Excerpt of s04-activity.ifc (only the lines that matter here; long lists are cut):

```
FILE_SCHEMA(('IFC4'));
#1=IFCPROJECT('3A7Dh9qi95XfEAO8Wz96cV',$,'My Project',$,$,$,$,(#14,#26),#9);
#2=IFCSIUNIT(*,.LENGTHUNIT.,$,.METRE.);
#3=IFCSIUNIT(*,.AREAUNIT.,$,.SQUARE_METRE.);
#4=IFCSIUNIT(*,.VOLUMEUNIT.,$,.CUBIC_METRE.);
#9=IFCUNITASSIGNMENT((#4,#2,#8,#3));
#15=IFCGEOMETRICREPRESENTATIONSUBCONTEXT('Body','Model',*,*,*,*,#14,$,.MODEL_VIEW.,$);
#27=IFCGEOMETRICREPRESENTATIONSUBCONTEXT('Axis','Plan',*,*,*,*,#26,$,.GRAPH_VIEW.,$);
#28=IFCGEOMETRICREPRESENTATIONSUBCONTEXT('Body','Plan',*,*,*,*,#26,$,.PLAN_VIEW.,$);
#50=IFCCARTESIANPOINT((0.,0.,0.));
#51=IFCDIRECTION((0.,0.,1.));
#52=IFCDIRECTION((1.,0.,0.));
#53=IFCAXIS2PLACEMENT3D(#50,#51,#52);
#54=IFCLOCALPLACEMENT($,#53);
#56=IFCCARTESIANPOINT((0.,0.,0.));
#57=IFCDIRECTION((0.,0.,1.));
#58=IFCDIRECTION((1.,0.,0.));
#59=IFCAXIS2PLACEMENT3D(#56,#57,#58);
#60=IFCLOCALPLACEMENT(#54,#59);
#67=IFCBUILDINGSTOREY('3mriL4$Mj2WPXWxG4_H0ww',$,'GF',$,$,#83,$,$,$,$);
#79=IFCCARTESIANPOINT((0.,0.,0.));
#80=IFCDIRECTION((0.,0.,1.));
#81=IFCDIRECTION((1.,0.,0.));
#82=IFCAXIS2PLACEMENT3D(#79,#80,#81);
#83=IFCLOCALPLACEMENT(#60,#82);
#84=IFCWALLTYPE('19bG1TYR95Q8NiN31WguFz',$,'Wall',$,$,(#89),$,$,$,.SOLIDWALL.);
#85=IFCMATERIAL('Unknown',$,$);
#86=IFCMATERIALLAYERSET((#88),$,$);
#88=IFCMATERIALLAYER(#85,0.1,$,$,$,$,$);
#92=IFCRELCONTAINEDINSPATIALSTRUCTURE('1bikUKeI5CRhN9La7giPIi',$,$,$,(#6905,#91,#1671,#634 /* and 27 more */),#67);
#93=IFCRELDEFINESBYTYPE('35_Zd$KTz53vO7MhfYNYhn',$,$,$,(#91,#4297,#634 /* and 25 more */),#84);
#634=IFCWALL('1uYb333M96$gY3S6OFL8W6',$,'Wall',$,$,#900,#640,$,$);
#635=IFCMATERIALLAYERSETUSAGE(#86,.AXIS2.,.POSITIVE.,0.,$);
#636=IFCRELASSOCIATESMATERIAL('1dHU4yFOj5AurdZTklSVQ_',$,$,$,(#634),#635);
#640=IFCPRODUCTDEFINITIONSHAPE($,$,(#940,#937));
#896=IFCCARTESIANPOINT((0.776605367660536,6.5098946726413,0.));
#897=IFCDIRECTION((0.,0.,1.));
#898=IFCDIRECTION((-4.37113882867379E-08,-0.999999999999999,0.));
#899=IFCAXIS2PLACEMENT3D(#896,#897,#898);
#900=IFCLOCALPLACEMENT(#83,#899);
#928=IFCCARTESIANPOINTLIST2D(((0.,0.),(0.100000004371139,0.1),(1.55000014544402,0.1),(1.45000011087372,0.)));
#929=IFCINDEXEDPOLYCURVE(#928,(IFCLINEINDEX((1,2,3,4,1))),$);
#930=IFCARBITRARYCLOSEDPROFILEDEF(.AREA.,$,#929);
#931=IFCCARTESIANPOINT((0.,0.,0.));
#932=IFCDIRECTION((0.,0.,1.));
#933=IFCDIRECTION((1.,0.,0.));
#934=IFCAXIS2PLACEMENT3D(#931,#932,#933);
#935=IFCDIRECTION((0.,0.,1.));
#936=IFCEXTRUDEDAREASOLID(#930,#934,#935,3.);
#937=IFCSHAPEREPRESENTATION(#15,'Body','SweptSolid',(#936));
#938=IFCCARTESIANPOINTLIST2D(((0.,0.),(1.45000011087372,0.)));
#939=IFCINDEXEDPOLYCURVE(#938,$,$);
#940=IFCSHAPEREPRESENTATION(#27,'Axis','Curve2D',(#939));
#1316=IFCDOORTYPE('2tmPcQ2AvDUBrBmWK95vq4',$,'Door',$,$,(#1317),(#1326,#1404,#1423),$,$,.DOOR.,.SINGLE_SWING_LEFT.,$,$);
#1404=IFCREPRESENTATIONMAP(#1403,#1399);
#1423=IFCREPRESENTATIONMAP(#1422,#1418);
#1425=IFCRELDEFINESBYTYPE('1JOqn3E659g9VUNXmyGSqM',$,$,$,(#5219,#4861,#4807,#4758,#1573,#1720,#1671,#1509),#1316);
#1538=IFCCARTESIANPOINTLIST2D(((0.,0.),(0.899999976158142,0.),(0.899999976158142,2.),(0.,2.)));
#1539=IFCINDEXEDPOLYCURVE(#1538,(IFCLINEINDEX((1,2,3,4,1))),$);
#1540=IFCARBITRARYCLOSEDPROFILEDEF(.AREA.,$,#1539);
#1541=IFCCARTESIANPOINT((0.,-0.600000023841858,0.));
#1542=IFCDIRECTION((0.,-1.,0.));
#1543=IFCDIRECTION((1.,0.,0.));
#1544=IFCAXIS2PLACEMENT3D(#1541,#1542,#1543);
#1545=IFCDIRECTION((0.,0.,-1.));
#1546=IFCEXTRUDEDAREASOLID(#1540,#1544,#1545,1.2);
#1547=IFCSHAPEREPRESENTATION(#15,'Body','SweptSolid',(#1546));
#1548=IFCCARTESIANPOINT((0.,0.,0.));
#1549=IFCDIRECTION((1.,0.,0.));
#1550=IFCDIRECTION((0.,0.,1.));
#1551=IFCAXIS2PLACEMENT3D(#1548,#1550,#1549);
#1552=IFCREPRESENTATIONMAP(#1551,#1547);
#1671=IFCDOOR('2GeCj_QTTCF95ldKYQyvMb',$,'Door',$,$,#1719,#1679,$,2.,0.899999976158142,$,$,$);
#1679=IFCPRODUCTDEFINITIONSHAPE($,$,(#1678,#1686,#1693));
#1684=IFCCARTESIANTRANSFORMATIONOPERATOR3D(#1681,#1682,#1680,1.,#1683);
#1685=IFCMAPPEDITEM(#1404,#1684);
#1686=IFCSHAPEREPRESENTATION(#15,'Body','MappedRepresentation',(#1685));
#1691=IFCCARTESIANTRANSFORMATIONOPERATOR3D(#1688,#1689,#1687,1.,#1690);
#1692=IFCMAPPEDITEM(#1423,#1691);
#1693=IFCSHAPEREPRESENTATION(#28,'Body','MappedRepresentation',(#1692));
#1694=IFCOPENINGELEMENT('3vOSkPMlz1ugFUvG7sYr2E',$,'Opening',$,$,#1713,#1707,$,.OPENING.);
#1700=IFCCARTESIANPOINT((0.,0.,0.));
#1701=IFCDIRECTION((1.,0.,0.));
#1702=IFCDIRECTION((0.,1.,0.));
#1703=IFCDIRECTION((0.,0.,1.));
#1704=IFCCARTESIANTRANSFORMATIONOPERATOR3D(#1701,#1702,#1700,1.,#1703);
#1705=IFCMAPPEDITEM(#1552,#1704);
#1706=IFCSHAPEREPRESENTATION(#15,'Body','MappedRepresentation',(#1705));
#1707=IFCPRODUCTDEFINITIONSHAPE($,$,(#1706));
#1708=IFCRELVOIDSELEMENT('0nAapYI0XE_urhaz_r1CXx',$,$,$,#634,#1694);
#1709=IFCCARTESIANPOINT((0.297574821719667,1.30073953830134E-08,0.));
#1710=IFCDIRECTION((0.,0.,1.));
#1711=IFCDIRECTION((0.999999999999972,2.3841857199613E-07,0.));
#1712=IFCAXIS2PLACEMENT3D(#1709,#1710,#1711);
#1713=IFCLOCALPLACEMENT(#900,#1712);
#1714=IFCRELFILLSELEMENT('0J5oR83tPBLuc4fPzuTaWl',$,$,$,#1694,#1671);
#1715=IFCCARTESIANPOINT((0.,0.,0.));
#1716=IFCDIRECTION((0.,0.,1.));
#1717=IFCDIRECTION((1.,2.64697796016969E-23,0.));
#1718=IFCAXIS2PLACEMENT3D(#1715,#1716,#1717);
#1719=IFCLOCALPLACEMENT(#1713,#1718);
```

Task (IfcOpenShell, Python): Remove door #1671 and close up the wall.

```python
import ifcopenshell
import ifcopenshell.api.feature
import ifcopenshell.api.root
import ifcopenshell.geom
import ifcopenshell.util.shape

model = ifcopenshell.open("s04-activity.ifc")
settings = ifcopenshell.geom.settings()


def volume(element):
    """Net volume in cubic metres, openings subtracted."""
    shape = ifcopenshell.geom.create_shape(settings, element)
    return ifcopenshell.util.shape.get_volume(shape.geometry)


door = model.by_guid("2GeCj_QTTCF95ldKYQyvMb")
opening = door.FillsVoids[0].RelatingOpeningElement
wall = opening.VoidsElements[0].RelatingBuildingElement
before = volume(wall)

ifcopenshell.api.root.remove_product(model, product=door)
ifcopenshell.api.feature.remove_feature(model, feature=opening)

after = volume(wall)

print(f"wall volume {before:.3f} -> {after:.3f} m3")

model.write("s04-activity_rev.ifc")
```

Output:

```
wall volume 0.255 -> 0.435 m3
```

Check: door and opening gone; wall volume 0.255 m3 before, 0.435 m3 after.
